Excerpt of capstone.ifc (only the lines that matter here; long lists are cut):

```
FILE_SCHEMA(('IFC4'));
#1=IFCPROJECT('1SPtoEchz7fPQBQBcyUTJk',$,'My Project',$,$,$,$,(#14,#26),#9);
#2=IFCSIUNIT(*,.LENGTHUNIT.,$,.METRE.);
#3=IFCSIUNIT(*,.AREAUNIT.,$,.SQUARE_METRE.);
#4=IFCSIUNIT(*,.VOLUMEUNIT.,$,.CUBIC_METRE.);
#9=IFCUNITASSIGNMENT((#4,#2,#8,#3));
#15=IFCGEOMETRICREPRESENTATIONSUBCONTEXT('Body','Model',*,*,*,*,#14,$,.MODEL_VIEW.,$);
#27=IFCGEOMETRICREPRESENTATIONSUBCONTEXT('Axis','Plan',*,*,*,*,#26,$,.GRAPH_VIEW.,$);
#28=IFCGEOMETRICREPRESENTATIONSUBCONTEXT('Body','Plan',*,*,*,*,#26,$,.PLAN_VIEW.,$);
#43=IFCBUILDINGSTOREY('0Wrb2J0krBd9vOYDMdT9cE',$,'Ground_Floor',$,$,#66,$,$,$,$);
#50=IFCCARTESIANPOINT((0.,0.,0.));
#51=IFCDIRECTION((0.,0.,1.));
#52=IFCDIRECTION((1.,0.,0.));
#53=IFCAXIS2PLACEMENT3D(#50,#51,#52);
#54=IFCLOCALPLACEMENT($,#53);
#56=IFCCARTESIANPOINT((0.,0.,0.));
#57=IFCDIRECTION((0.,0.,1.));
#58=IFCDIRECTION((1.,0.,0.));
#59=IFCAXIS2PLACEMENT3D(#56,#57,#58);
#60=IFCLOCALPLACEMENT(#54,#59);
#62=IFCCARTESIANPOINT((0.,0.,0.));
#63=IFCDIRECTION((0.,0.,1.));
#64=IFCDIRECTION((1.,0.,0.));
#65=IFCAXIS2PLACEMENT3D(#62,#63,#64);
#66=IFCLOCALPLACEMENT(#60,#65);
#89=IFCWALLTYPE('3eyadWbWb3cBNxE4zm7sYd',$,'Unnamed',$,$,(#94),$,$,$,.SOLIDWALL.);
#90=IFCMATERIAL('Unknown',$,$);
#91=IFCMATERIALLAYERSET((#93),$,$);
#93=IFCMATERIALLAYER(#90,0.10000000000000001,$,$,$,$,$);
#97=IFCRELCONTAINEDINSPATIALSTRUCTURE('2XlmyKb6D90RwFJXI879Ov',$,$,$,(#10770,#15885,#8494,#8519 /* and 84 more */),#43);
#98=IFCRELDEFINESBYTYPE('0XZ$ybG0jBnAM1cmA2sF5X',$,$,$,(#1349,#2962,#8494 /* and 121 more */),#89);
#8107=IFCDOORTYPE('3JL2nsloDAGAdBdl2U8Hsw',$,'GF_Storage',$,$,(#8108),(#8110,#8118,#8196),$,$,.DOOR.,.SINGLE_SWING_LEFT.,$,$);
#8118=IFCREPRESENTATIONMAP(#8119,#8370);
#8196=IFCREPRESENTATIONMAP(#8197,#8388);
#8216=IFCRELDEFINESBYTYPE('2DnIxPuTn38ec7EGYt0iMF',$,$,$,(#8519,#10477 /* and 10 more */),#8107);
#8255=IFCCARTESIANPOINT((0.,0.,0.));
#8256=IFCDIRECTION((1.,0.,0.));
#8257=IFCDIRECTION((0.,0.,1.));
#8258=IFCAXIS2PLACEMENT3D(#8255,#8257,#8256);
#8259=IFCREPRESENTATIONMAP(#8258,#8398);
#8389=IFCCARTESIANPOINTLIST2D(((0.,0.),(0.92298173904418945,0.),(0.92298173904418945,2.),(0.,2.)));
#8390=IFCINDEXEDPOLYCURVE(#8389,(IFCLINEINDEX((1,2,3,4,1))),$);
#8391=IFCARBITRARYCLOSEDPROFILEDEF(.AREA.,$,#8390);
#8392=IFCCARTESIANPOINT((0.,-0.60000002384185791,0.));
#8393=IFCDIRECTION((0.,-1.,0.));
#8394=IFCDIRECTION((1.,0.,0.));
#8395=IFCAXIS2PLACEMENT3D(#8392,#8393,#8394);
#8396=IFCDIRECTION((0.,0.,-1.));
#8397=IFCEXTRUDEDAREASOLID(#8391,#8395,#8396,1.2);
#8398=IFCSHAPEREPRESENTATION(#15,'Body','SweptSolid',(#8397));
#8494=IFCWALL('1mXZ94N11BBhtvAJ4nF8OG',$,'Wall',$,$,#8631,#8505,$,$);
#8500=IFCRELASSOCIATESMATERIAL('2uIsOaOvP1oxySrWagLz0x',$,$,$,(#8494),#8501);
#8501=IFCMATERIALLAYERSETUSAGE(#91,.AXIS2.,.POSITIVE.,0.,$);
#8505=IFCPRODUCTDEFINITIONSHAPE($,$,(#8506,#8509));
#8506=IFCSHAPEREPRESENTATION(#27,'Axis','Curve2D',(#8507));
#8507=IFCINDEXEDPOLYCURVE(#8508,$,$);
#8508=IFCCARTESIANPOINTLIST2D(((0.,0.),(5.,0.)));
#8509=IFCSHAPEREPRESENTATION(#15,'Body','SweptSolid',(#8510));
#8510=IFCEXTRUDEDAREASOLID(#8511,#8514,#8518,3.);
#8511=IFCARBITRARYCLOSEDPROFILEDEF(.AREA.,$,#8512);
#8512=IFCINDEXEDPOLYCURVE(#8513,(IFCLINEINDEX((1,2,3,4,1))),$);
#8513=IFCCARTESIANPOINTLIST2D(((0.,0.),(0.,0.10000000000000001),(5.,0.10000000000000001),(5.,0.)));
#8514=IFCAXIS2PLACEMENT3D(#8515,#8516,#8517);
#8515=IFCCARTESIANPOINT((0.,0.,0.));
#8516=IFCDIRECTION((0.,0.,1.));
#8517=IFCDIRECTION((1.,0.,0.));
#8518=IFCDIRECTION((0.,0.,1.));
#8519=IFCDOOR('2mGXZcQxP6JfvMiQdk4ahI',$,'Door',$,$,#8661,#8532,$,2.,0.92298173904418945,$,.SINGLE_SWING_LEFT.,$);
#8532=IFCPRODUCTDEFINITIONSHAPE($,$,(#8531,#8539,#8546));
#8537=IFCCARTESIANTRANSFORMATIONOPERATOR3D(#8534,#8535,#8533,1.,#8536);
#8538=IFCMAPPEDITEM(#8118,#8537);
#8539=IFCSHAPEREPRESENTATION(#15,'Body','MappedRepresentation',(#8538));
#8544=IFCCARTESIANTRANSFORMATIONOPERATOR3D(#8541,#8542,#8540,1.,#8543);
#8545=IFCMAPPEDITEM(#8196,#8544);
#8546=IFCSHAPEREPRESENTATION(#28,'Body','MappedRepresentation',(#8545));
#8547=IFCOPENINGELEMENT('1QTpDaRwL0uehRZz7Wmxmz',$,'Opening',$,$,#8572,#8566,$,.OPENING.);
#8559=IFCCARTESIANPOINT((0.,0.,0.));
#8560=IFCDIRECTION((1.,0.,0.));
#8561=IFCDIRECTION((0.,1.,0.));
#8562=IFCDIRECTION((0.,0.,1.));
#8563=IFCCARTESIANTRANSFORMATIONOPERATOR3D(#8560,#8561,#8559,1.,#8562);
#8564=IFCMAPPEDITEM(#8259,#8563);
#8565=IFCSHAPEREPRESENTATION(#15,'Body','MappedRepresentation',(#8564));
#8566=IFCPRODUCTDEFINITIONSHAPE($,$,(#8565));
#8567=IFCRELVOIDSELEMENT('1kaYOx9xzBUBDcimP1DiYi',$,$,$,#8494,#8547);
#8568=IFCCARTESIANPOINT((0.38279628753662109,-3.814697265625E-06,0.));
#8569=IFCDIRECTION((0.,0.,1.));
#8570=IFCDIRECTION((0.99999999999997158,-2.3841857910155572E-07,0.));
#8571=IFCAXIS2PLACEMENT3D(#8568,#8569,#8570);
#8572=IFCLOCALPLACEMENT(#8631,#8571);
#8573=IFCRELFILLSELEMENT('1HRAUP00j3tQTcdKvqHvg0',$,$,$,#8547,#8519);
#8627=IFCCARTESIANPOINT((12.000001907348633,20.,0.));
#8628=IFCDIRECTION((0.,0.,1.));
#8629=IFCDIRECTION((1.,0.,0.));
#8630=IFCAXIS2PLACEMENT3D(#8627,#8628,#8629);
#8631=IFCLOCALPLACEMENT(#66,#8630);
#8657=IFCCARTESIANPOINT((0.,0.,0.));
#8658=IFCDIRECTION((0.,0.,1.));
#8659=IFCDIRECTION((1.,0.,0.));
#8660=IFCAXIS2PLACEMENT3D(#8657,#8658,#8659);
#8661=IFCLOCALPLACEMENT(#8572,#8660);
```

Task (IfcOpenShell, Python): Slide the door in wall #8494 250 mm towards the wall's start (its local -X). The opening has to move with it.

```python
import ifcopenshell
import ifcopenshell.api.geometry
import ifcopenshell.util.placement
import ifcopenshell.util.unit

model = ifcopenshell.open("capstone.ifc")
unit_scale = ifcopenshell.util.unit.calculate_unit_scale(model)

door = model.by_guid("2mGXZcQxP6JfvMiQdk4ahI")
opening = door.FillsVoids[0].RelatingOpeningElement
wall = opening.VoidsElements[0].RelatingBuildingElement

wall_matrix = ifcopenshell.util.placement.get_local_placement(wall.ObjectPlacement)
shift = wall_matrix[:3, 0] * -0.25 / unit_scale
before = ifcopenshell.util.placement.get_local_placement(door.ObjectPlacement)[:3, 3].copy()

# The door is placed relative to its opening, so it follows when the opening moves.
matrix = ifcopenshell.util.placement.get_local_placement(opening.ObjectPlacement)
matrix[:3, 3] += shift
ifcopenshell.api.geometry.edit_object_placement(
    model, product=opening, matrix=matrix, is_si=False, should_transform_children=True
)

after = ifcopenshell.util.placement.get_local_placement(door.ObjectPlacement)[:3, 3]
print("door moved by", (after - before).round(3) + 0.0)

model.write("capstone_edited.ifc")
```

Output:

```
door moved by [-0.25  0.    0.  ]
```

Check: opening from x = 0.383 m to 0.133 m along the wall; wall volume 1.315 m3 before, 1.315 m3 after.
